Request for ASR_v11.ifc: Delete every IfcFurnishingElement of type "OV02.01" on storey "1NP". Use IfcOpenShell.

First a look at what the model holds.

```python
import ifcopenshell
import ifcopenshell.util.element

model = ifcopenshell.open("ASR_v11.ifc")
print(model.schema)
storey = next(s for s in model.by_type("IfcBuildingStorey") if s.Name == "1NP")
furniture = [e for e in ifcopenshell.util.element.get_decomposition(storey) if e.is_a("IfcFurnishingElement")]
seen = {}
for e in furniture:
    element_type = ifcopenshell.util.element.get_type(e)
    name = element_type.Name if element_type not in (None, e) else None
    seen[name] = seen.get(name, 0) + 1
for name, count in sorted(seen.items(), key=str):
    print(count, "x", name)
```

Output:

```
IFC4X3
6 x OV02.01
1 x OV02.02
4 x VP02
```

```python
import ifcopenshell
import ifcopenshell.api.root
import ifcopenshell.util.element

model = ifcopenshell.open("ASR_v11.ifc")

storey = next(s for s in model.by_type("IfcBuildingStorey") if s.Name == "1NP")
furniture = [e for e in ifcopenshell.util.element.get_decomposition(storey) if e.is_a("IfcFurnishingElement")]
targets = [e for e in furniture if (t := ifcopenshell.util.element.get_type(e)) not in (None, e) and t.Name == "OV02.01"]

for e in targets:
    ifcopenshell.api.root.remove_product(model, product=e)
print(len(targets), "removed")

model.write("ASR_v11_rev.ifc")
```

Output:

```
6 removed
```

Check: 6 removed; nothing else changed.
